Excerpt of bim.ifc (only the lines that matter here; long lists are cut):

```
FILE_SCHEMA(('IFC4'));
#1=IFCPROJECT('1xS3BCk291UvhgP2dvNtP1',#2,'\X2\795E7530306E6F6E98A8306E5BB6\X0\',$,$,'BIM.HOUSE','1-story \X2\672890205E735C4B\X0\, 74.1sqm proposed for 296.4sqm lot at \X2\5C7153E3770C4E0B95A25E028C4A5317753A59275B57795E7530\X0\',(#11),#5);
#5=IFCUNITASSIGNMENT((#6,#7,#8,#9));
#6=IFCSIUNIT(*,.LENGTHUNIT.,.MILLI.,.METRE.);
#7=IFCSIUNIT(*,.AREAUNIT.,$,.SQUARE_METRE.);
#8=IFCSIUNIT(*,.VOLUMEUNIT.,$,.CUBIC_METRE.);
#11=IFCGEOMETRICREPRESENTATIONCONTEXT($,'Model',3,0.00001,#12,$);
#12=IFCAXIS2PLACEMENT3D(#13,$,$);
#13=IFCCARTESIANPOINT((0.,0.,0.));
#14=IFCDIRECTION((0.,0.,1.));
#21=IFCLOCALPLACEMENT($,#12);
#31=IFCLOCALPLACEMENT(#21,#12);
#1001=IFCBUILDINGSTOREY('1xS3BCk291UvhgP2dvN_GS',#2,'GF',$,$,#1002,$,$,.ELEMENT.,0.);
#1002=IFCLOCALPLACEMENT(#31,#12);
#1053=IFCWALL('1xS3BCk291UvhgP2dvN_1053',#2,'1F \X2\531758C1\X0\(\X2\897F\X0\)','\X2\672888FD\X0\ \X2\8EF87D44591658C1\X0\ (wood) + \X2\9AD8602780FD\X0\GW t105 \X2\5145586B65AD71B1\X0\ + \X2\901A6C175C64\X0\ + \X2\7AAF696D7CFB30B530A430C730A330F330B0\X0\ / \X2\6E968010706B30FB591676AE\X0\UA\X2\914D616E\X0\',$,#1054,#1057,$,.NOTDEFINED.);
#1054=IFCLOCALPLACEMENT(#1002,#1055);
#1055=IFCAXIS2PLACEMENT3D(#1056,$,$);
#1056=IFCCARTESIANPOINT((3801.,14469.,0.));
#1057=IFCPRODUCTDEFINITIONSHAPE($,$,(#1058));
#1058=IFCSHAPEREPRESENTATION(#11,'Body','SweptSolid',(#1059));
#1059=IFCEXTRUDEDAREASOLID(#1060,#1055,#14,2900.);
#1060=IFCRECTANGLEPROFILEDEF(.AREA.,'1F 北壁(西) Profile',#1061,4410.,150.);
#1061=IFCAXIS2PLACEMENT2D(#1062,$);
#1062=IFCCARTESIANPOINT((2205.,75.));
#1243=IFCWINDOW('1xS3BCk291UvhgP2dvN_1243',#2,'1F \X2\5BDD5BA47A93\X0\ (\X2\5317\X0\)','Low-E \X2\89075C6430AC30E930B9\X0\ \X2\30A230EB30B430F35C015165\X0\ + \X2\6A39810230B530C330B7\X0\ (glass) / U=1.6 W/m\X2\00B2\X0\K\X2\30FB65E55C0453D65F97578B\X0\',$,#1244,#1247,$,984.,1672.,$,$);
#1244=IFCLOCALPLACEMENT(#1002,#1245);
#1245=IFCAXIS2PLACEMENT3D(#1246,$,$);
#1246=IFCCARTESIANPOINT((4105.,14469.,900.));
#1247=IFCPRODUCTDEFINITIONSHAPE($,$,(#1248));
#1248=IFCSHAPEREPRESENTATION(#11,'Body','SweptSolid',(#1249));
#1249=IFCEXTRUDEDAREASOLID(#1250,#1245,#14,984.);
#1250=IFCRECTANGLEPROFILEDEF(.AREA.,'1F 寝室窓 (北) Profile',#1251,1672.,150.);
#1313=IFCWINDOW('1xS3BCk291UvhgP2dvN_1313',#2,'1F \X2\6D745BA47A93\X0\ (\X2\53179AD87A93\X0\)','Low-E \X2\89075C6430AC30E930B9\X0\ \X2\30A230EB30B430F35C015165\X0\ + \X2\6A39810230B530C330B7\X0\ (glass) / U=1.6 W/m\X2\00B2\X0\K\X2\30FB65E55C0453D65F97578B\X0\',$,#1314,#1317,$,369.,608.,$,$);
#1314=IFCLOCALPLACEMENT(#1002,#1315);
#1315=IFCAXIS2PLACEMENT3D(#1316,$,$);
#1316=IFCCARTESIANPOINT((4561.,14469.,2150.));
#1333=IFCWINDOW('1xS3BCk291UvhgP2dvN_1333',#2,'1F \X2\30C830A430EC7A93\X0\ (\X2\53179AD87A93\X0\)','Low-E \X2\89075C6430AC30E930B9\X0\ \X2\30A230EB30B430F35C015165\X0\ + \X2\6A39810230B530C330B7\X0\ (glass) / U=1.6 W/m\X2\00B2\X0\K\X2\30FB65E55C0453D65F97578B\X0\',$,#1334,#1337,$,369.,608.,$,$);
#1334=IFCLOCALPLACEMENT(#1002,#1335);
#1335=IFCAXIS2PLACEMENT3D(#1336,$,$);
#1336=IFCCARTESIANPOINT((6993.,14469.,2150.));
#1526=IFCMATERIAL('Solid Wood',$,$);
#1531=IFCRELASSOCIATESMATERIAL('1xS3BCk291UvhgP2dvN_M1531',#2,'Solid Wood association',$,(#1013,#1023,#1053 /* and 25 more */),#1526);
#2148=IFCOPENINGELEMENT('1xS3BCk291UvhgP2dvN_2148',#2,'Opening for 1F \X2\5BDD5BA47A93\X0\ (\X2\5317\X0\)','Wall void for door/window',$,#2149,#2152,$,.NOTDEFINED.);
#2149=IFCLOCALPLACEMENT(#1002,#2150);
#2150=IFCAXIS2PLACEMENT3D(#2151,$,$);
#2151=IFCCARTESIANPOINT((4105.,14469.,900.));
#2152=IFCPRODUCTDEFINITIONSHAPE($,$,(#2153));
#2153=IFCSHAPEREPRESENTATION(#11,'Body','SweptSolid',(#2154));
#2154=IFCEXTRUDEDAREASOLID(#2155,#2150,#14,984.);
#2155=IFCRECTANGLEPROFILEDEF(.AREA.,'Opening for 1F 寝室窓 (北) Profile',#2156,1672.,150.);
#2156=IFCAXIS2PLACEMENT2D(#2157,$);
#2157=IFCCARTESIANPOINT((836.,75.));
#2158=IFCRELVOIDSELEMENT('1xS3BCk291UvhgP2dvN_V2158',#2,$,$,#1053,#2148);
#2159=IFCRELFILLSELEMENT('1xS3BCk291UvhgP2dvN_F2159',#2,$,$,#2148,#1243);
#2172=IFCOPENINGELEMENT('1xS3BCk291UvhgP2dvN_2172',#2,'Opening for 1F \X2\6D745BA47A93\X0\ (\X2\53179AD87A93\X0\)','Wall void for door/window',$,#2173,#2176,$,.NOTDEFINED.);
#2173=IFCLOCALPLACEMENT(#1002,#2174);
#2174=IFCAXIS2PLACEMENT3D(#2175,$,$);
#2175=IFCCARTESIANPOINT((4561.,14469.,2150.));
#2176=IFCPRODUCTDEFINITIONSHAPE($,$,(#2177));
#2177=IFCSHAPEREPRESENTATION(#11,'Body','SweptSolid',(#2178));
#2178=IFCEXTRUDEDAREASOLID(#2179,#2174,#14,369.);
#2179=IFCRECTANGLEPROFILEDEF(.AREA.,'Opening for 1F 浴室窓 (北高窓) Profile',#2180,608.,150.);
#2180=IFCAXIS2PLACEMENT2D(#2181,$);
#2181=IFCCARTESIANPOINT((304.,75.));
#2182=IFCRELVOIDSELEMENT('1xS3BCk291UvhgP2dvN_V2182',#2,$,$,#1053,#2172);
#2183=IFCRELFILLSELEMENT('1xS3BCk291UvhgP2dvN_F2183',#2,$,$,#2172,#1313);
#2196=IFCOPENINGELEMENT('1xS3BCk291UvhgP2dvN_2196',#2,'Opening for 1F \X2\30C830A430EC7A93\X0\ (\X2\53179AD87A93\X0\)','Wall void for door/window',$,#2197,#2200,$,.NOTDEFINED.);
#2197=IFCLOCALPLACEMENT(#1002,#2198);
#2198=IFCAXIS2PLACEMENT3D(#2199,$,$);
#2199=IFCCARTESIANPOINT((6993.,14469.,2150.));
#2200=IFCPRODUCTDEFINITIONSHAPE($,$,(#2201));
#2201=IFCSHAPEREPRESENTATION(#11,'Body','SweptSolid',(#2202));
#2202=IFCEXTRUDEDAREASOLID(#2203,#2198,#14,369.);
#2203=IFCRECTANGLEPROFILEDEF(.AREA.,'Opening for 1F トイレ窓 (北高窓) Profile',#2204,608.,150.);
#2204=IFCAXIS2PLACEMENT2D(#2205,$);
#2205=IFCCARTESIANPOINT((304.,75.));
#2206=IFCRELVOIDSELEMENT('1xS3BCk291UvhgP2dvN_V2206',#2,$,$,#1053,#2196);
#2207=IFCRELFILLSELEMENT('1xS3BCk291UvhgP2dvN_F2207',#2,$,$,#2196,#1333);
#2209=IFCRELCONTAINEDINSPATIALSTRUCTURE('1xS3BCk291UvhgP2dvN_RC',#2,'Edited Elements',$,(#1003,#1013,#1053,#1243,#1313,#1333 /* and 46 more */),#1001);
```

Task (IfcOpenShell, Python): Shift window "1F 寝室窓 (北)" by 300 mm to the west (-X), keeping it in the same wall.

```python
import ifcopenshell
import ifcopenshell.api.geometry
import ifcopenshell.util.placement

model = ifcopenshell.open("bim.ifc")

window = model.by_guid("1xS3BCk291UvhgP2dvN_1243")
opening = window.FillsVoids[0].RelatingOpeningElement
wall = opening.VoidsElements[0].RelatingBuildingElement

wall_matrix = ifcopenshell.util.placement.get_local_placement(wall.ObjectPlacement)
shift = wall_matrix[:3, 0] * -300.0
before = ifcopenshell.util.placement.get_local_placement(window.ObjectPlacement)[:3, 3].copy()

# The window is not placed relative to its opening, so move both.
for product in (opening, window):
    matrix = ifcopenshell.util.placement.get_local_placement(product.ObjectPlacement)
    matrix[:3, 3] += shift
    ifcopenshell.api.geometry.edit_object_placement(model, product=product, matrix=matrix, is_si=False)

after = ifcopenshell.util.placement.get_local_placement(window.ObjectPlacement)[:3, 3]
print("window moved by", (after - before).round(3) + 0.0)

model.write("bim_updated.ifc")
```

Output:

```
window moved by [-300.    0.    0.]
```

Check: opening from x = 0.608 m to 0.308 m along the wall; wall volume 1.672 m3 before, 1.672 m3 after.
